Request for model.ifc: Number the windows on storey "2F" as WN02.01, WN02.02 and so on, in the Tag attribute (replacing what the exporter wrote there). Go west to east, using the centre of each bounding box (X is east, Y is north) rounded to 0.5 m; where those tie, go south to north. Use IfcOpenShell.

First a look at what the model holds.

```python
import ifcopenshell
import ifcopenshell.util.element
import ifcopenshell.util.placement

model = ifcopenshell.open("model.ifc")
print(model.schema)
storey = next(s for s in model.by_type("IfcBuildingStorey") if s.Name == "2F")
windows = [e for e in ifcopenshell.util.element.get_decomposition(storey) if e.is_a("IfcWindow")]
for e in sorted(windows, key=lambda e: e.id()):
    origin = ifcopenshell.util.placement.get_local_placement(e.ObjectPlacement)[:3, 3]
    print(e.id(), e.Tag, e.Name, origin.round(2) + 0.0, sep=" | ")
```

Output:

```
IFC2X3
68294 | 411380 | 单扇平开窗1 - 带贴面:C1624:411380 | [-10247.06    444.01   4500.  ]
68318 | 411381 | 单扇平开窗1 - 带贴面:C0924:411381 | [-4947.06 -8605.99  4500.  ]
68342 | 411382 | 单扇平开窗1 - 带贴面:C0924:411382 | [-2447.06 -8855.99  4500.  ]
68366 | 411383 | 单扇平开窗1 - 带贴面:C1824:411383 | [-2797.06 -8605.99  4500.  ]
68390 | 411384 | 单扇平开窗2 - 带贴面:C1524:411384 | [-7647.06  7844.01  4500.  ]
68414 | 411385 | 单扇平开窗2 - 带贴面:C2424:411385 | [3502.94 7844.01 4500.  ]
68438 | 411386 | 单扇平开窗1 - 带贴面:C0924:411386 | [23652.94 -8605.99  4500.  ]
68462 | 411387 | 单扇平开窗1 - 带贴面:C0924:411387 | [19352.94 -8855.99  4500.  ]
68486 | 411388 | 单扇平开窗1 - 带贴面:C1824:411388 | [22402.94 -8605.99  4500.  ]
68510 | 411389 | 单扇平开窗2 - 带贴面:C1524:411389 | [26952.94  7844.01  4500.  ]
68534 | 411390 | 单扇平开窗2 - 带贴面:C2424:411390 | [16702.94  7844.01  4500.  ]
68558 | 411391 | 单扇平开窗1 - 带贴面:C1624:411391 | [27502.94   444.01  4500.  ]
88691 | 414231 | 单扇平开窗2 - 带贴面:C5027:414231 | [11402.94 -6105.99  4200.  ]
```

```python
import ifcopenshell
import ifcopenshell.geom
import ifcopenshell.util.element
import ifcopenshell.util.shape

model = ifcopenshell.open("model.ifc")
settings = ifcopenshell.geom.settings()
settings.set("use-world-coords", True)


def centre(element):
    shape = ifcopenshell.geom.create_shape(settings, element)
    return ifcopenshell.util.shape.get_bbox_centroid(shape.geometry)


storey = next(s for s in model.by_type("IfcBuildingStorey") if s.Name == "2F")
windows = [e for e in ifcopenshell.util.element.get_decomposition(storey) if e.is_a("IfcWindow")]

# Insertion points can sit at a corner or the storey origin, so sort by the geometry (in metres).
centres = {e: centre(e) for e in windows}
windows.sort(key=lambda e: (round(centres[e][0] / 0.5), centres[e][1]))

for i, e in enumerate(windows, start=1):
    number = f"WN02.{i:02d}"
    e.Tag = number
    print(e.id(), number)

model.write("model_updated.ifc")
```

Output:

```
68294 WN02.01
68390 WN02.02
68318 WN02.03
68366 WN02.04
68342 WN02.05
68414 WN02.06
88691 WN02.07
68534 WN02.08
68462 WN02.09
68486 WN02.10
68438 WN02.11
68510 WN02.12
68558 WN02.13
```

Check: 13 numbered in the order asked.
